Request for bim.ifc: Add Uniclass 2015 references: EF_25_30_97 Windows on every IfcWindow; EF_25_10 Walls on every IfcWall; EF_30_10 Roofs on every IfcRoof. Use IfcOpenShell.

First a look at what the model holds.

```python
import ifcopenshell

model = ifcopenshell.open("bim.ifc")
print(model.schema)
print("classifications:", [c.Name for c in model.by_type("IfcClassification")])
for ifc_class in ("IfcDoor", "IfcRoof", "IfcStair", "IfcWall", "IfcWindow"):
    print(ifc_class, len(model.by_type(ifc_class)))
```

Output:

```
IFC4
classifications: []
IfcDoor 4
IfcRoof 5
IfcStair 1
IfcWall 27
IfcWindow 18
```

```python
import ifcopenshell
import ifcopenshell.api.classification

model = ifcopenshell.open("bim.ifc")

system = ifcopenshell.api.classification.add_classification(model, classification="Uniclass 2015")

codes = {
    "IfcWindow": ("EF_25_30_97", "Windows"),
    "IfcWall": ("EF_25_10", "Walls"),
    "IfcRoof": ("EF_30_10", "Roofs"),
}
for ifc_class, (code, name) in codes.items():
    products = model.by_type(ifc_class)
    ifcopenshell.api.classification.add_reference(
        model, products=products, classification=system, identification=code, name=name
    )
    print(code, len(products))

model.write("bim-out.ifc")
```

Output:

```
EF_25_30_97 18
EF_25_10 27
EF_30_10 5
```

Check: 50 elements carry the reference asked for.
